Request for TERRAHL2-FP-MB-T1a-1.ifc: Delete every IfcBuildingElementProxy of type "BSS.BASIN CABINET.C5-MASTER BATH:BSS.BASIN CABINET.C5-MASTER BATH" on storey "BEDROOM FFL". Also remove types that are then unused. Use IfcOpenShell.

First a look at what the model holds.

```python
import ifcopenshell
import ifcopenshell.util.element

model = ifcopenshell.open("TERRAHL2-FP-MB-T1a-1.ifc")
print(model.schema)
storey = next(s for s in model.by_type("IfcBuildingStorey") if s.Name == "BEDROOM FFL")
proxies = [e for e in ifcopenshell.util.element.get_decomposition(storey) if e.is_a("IfcBuildingElementProxy")]
seen = {}
for e in proxies:
    element_type = ifcopenshell.util.element.get_type(e)
    name = element_type.Name if element_type not in (None, e) else None
    seen[name] = seen.get(name, 0) + 1
for name, count in sorted(seen.items(), key=str):
    print(count, "x", name)
```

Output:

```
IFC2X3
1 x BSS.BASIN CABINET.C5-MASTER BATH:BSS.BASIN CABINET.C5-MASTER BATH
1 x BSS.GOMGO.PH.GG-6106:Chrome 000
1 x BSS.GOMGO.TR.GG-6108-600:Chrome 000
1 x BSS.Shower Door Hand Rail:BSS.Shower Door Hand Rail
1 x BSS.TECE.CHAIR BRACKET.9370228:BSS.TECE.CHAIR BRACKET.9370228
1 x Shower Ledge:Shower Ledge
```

```python
import ifcopenshell
import ifcopenshell.api.root
import ifcopenshell.util.element

model = ifcopenshell.open("TERRAHL2-FP-MB-T1a-1.ifc")

storey = next(s for s in model.by_type("IfcBuildingStorey") if s.Name == "BEDROOM FFL")
proxies = [e for e in ifcopenshell.util.element.get_decomposition(storey) if e.is_a("IfcBuildingElementProxy")]
targets = [e for e in proxies if (t := ifcopenshell.util.element.get_type(e)) not in (None, e) and t.Name == "BSS.BASIN CABINET.C5-MASTER BATH:BSS.BASIN CABINET.C5-MASTER BATH"]
types = {ifcopenshell.util.element.get_type(e) for e in targets} - {None, *targets}

for e in targets:
    ifcopenshell.api.root.remove_product(model, product=e)
print(len(targets), "removed")

unused = [t for t in types if not ifcopenshell.util.element.get_types(t)]
for t in unused:
    ifcopenshell.api.root.remove_product(model, product=t)
print(len(unused), "unused types removed")

model.write("TERRAHL2-FP-MB-T1a-1_v2.ifc")
```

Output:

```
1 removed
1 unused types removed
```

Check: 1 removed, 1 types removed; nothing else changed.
